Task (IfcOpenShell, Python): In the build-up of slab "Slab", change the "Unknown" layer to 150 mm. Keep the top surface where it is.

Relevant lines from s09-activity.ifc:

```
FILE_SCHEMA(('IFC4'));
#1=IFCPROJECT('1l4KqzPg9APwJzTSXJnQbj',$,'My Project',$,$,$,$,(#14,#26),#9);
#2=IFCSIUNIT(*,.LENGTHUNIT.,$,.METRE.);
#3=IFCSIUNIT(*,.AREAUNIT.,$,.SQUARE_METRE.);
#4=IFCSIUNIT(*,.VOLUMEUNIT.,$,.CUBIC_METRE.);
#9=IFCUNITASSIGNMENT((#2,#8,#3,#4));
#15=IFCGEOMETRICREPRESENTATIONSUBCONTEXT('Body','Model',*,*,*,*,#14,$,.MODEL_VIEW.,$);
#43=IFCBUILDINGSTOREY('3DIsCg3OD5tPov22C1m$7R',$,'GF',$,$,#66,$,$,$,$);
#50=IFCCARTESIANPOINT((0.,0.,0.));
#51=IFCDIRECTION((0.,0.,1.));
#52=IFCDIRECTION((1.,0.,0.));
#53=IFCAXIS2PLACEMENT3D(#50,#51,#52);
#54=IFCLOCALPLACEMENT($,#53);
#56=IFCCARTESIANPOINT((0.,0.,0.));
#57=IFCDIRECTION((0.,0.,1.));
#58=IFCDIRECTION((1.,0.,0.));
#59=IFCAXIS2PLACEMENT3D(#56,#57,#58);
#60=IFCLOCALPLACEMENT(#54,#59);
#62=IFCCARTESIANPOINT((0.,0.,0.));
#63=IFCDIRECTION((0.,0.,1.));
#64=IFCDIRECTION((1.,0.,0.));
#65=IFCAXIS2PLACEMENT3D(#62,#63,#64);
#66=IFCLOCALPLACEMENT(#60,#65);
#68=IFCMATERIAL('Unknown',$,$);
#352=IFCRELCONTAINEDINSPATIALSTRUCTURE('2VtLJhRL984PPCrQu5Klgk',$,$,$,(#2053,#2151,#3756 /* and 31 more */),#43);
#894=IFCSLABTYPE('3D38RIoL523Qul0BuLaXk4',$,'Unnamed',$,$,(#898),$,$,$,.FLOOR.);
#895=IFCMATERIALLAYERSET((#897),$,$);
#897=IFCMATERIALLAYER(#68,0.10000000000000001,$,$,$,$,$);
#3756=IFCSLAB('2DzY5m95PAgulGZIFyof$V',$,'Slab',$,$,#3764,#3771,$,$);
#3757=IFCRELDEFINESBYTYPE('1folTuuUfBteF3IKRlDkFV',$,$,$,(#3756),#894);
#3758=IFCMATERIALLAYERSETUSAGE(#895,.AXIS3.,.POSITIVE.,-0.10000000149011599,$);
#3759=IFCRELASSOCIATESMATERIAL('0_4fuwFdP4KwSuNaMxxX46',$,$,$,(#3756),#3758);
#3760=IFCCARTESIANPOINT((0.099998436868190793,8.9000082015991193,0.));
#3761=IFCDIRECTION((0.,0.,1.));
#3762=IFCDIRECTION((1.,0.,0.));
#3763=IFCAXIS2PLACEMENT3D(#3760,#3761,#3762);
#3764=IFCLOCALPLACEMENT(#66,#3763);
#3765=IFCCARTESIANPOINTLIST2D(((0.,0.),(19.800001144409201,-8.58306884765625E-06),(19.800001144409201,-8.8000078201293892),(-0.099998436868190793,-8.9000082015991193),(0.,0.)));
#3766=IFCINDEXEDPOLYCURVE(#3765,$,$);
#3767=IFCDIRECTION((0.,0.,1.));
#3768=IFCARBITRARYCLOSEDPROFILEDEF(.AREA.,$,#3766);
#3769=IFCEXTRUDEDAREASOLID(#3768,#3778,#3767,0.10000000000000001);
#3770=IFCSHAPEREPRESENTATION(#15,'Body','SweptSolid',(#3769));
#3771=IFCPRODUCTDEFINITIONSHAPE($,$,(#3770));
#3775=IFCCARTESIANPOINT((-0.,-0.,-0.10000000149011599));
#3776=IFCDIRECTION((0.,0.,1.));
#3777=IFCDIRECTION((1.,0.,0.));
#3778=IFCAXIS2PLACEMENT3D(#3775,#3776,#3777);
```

```python
import ifcopenshell
import ifcopenshell.util.element
import ifcopenshell.util.representation

model = ifcopenshell.open("s09-activity.ifc")

layer_set = model.by_id(895)
layer = next(l for l in layer_set.MaterialLayers if l.Material and l.Material.Name == "Unknown")
change = 0.15 - layer.LayerThickness
layer.LayerThickness += change

# Geometry does not follow the layer set by itself.
slabs = [e for e in ifcopenshell.util.element.get_elements_by_material(model, layer_set) if e.is_a("IfcSlab")]
for slab in sorted(slabs, key=lambda e: e.id()):
    body = ifcopenshell.util.representation.get_representation(slab, "Model", "Body")
    solid = body.Items[0]
    old_depth = solid.Depth
    solid.Depth += change
    # Extruded upwards: lower the start of the extrusion so the top stays.
    x, y, z = solid.Position.Location.Coordinates
    solid.Position.Location = model.createIfcCartesianPoint((x, y, z - change))
    print(slab.id(), f"{old_depth:g} -> {solid.Depth:g}")

# The layers are counted up from the underside, which has moved.
for usage in {ifcopenshell.util.element.get_material(slab) for slab in slabs}:
    usage.OffsetFromReferenceLine -= change

model.write("s09-activity_edited.ifc")
```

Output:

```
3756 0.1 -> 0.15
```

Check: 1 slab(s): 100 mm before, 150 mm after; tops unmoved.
